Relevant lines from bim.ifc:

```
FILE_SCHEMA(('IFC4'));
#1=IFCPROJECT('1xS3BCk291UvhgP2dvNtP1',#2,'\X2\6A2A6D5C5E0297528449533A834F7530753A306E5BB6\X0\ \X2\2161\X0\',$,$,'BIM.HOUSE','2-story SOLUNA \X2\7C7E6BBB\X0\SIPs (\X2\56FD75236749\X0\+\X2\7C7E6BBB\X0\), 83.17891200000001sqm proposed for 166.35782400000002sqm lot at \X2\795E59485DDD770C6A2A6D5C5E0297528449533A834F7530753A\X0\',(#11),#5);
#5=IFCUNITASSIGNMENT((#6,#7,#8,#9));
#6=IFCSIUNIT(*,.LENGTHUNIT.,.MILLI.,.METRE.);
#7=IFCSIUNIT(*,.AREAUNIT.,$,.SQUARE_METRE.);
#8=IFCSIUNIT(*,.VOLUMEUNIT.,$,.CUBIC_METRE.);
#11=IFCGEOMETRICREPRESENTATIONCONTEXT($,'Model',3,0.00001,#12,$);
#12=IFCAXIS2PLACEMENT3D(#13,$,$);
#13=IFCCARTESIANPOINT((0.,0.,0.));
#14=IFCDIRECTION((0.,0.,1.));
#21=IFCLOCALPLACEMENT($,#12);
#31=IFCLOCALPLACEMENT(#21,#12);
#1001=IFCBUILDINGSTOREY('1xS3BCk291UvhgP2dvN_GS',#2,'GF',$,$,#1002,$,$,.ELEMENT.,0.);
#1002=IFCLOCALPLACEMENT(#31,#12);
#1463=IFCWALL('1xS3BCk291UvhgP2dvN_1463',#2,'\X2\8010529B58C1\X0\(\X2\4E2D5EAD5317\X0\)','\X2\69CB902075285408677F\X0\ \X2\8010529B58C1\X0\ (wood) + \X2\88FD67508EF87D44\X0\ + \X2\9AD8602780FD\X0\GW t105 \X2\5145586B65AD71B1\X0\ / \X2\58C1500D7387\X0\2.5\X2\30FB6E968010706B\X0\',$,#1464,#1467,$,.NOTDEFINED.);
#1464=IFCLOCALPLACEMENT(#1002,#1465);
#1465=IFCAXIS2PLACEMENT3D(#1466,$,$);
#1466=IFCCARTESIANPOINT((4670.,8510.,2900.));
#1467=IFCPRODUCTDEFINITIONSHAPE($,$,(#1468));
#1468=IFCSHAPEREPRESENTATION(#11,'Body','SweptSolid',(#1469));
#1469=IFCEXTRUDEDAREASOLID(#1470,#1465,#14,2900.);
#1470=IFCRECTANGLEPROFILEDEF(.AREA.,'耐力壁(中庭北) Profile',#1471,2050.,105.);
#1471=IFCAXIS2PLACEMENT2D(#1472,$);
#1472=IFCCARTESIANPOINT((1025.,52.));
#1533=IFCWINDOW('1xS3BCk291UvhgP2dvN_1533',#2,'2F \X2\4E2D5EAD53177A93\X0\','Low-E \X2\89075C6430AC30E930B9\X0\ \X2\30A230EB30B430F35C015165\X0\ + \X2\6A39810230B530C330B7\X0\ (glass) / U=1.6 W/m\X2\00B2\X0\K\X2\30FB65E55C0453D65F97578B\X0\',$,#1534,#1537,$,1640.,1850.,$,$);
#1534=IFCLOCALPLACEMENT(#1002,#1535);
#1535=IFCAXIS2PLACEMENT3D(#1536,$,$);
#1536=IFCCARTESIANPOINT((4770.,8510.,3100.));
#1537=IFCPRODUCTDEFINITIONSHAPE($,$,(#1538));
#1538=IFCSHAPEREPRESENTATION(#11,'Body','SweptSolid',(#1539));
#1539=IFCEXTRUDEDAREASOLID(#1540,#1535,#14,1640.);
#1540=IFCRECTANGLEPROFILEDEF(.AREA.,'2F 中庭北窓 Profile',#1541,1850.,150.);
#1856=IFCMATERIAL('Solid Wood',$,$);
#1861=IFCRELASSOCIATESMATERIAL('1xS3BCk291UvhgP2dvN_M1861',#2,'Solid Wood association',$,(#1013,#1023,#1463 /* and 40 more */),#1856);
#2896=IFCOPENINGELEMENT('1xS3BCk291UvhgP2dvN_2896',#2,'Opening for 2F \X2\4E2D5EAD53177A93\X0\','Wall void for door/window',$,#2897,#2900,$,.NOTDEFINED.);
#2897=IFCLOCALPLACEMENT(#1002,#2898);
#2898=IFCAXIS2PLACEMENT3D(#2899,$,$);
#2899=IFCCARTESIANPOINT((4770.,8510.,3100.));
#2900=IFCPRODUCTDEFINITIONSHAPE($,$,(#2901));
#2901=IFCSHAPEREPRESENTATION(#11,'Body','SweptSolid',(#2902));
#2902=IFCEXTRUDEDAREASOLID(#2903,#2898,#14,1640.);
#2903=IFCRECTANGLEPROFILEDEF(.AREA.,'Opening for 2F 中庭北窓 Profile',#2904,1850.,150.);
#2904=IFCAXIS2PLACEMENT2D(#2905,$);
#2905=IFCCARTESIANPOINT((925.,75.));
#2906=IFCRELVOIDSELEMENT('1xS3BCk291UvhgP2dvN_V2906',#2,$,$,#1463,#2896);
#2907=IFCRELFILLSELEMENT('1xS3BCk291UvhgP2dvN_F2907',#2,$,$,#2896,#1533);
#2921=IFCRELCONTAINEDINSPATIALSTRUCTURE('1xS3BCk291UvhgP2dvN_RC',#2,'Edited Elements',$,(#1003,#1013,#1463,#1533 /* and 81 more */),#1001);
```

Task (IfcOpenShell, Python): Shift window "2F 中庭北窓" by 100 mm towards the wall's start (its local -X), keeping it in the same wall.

```python
import ifcopenshell
import ifcopenshell.api.geometry
import ifcopenshell.util.placement
import ifcopenshell.util.unit

model = ifcopenshell.open("bim.ifc")
unit_scale = ifcopenshell.util.unit.calculate_unit_scale(model)

window = model.by_guid("1xS3BCk291UvhgP2dvN_1533")
opening = window.FillsVoids[0].RelatingOpeningElement
wall = opening.VoidsElements[0].RelatingBuildingElement

wall_matrix = ifcopenshell.util.placement.get_local_placement(wall.ObjectPlacement)
shift = wall_matrix[:3, 0] * -0.1 / unit_scale
before = ifcopenshell.util.placement.get_local_placement(window.ObjectPlacement)[:3, 3].copy()

# The window is not placed relative to its opening, so move both.
for product in (opening, window):
    matrix = ifcopenshell.util.placement.get_local_placement(product.ObjectPlacement)
    matrix[:3, 3] += shift
    ifcopenshell.api.geometry.edit_object_placement(model, product=product, matrix=matrix, is_si=False)

after = ifcopenshell.util.placement.get_local_placement(window.ObjectPlacement)[:3, 3]
print("window moved by", (after - before).round(3) + 0.0)

model.write("bim-out.ifc")
```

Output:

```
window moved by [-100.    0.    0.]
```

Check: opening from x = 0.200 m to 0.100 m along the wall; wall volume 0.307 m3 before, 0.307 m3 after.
